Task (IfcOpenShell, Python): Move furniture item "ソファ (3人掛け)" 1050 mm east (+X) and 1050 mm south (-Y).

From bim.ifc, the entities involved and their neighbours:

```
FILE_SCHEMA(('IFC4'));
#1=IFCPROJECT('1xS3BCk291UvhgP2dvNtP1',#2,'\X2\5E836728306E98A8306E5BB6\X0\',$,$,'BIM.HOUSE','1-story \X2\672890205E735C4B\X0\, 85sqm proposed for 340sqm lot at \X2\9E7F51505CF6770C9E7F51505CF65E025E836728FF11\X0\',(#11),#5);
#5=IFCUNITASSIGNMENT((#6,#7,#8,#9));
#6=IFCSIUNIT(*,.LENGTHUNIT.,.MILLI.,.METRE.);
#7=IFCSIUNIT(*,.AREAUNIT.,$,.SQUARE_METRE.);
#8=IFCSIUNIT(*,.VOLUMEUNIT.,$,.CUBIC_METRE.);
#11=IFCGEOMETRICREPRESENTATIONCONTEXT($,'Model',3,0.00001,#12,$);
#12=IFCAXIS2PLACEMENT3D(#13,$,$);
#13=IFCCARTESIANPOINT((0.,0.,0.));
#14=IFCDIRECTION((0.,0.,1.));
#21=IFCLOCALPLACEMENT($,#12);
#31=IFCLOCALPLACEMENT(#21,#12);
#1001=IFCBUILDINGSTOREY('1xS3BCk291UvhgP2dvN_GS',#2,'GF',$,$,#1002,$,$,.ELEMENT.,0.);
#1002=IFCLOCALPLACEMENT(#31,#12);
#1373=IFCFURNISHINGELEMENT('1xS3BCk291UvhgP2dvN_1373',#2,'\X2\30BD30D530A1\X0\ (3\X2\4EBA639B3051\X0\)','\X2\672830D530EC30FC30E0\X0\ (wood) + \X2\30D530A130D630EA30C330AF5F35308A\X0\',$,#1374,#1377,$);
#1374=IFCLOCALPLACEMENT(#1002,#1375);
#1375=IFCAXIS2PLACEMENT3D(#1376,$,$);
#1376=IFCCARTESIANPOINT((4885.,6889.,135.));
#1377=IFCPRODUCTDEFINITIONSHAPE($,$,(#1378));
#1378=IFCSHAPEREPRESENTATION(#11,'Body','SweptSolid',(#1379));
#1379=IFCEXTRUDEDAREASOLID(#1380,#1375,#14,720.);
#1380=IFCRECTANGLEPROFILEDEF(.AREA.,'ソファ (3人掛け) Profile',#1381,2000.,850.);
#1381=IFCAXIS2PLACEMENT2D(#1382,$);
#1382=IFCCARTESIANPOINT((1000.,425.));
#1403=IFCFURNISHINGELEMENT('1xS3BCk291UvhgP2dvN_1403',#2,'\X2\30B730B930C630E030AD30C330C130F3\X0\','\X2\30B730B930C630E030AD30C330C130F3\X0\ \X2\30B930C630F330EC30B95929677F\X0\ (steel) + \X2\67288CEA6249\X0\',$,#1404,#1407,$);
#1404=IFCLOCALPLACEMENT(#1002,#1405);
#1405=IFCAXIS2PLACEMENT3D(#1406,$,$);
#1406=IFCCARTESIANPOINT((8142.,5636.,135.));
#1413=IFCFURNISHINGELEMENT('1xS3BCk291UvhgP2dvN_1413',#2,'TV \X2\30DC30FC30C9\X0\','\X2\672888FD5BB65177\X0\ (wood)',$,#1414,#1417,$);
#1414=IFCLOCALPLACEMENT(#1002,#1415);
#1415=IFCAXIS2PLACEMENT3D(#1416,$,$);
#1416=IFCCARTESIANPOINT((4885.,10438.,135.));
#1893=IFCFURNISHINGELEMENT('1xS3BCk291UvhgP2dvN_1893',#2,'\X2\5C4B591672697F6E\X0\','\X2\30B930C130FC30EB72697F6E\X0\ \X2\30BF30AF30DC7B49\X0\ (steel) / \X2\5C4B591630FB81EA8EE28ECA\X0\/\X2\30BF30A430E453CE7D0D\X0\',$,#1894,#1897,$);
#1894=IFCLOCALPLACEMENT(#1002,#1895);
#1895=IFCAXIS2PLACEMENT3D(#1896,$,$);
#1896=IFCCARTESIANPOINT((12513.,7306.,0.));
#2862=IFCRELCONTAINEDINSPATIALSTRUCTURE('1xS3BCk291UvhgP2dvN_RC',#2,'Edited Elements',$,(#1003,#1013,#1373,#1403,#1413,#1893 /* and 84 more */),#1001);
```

```python
import ifcopenshell
import ifcopenshell.api.geometry
import ifcopenshell.util.placement

model = ifcopenshell.open("bim.ifc")

item = model.by_guid("1xS3BCk291UvhgP2dvN_1373")
matrix = ifcopenshell.util.placement.get_local_placement(item.ObjectPlacement)
matrix[0, 3] += 1050.0
matrix[1, 3] -= 1050.0
ifcopenshell.api.geometry.edit_object_placement(model, product=item, matrix=matrix, is_si=False)

print(ifcopenshell.util.placement.get_local_placement(item.ObjectPlacement).round(3) + 0.0)

model.write("bim_edited.ifc")
```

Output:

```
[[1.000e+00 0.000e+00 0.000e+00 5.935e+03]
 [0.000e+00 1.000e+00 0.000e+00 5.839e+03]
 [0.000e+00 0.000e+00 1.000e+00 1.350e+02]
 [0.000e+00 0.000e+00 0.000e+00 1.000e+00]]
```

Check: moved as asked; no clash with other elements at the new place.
